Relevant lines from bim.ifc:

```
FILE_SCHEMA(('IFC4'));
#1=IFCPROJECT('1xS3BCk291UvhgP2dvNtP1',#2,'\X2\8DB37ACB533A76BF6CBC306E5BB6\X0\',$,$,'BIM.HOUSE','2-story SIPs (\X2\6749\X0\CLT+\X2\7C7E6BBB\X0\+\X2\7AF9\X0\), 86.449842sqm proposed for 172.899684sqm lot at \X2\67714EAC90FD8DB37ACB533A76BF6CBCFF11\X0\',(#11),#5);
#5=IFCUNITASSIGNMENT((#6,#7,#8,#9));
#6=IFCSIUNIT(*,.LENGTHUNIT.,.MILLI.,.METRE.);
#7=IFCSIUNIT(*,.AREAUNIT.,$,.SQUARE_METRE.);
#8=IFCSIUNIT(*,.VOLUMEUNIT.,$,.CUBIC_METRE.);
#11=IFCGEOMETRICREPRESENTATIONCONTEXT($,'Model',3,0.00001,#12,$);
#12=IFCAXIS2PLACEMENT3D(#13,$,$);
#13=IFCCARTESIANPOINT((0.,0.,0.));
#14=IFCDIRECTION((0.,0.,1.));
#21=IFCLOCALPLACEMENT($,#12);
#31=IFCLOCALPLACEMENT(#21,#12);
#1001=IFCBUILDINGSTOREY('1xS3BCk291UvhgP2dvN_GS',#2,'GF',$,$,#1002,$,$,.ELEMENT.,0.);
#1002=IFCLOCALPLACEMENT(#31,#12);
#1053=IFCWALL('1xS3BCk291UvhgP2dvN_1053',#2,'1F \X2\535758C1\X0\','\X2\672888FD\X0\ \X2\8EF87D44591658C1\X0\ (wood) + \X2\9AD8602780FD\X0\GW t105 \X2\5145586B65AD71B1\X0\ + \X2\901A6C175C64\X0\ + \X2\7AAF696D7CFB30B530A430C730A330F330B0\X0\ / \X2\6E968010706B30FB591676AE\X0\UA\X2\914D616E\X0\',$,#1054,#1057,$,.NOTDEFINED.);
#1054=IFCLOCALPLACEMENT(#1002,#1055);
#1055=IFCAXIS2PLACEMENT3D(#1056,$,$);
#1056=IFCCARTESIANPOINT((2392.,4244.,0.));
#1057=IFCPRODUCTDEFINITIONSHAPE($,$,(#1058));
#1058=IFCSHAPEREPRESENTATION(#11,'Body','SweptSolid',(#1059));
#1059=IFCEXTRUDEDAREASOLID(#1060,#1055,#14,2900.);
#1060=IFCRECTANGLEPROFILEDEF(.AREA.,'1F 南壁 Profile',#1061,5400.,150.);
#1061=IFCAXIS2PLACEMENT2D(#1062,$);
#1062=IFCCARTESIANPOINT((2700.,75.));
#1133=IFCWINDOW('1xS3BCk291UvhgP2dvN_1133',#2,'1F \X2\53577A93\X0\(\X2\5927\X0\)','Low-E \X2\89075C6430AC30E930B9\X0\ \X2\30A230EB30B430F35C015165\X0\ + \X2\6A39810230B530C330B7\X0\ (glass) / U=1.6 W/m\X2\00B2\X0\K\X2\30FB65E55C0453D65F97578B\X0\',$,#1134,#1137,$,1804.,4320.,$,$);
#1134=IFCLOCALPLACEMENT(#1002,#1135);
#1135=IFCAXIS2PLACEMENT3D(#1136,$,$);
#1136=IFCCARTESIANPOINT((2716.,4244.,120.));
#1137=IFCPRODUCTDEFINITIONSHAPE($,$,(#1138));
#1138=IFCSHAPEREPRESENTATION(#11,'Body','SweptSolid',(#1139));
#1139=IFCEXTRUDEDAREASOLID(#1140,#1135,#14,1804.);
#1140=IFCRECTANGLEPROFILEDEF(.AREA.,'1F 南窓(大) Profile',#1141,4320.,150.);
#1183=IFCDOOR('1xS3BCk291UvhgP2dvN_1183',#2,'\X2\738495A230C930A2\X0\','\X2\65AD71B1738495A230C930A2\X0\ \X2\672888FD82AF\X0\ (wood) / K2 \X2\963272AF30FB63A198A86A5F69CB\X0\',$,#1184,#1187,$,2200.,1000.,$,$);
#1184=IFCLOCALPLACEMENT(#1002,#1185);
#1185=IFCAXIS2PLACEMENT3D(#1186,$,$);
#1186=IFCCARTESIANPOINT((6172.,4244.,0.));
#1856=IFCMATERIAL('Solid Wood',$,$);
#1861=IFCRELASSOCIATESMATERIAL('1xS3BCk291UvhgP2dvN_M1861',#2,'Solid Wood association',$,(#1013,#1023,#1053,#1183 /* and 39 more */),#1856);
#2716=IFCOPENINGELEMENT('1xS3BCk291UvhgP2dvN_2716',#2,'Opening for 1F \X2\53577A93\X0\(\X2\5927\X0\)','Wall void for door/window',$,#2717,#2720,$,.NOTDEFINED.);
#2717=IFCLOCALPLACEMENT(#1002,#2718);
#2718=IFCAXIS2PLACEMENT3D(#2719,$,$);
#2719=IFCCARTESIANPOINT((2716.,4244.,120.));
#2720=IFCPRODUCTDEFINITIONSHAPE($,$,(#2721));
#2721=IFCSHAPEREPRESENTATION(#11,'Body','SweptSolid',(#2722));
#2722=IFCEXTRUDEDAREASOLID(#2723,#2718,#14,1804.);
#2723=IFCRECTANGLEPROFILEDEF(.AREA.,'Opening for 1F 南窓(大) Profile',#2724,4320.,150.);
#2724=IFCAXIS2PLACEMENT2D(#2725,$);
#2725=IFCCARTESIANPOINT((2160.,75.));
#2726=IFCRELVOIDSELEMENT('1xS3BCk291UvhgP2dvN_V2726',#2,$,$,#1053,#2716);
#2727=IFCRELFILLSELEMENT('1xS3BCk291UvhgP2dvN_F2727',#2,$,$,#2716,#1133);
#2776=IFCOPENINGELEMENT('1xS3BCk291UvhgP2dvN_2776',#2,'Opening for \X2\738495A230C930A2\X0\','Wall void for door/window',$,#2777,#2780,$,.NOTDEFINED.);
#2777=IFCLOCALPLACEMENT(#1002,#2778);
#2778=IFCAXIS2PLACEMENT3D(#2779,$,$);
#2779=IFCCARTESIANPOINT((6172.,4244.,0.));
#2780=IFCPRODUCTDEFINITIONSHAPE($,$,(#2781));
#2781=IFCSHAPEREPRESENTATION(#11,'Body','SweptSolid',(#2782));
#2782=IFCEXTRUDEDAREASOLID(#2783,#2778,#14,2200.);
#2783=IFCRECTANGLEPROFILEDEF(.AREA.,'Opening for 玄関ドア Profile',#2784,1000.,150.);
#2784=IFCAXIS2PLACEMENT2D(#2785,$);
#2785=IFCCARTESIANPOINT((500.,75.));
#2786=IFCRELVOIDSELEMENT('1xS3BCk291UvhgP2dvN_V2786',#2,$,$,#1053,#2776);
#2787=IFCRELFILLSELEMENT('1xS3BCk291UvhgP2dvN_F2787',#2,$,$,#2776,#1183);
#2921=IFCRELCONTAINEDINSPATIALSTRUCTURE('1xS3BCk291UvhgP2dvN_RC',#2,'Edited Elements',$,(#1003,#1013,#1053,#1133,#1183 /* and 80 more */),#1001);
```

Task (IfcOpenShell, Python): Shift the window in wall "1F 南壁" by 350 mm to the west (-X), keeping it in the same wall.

```python
import ifcopenshell
import ifcopenshell.api.geometry
import ifcopenshell.util.placement

model = ifcopenshell.open("bim.ifc")

window = model.by_guid("1xS3BCk291UvhgP2dvN_1133")
opening = window.FillsVoids[0].RelatingOpeningElement
wall = opening.VoidsElements[0].RelatingBuildingElement

wall_matrix = ifcopenshell.util.placement.get_local_placement(wall.ObjectPlacement)
shift = wall_matrix[:3, 0] * -350.0
before = ifcopenshell.util.placement.get_local_placement(window.ObjectPlacement)[:3, 3].copy()

# The window is not placed relative to its opening, so move both.
for product in (opening, window):
    matrix = ifcopenshell.util.placement.get_local_placement(product.ObjectPlacement)
    matrix[:3, 3] += shift
    ifcopenshell.api.geometry.edit_object_placement(model, product=product, matrix=matrix, is_si=False)

after = ifcopenshell.util.placement.get_local_placement(window.ObjectPlacement)[:3, 3]
print("window moved by", (after - before).round(3) + 0.0)

model.write("bim_v2.ifc")
```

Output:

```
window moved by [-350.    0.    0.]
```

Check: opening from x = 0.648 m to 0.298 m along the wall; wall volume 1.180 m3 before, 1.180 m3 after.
